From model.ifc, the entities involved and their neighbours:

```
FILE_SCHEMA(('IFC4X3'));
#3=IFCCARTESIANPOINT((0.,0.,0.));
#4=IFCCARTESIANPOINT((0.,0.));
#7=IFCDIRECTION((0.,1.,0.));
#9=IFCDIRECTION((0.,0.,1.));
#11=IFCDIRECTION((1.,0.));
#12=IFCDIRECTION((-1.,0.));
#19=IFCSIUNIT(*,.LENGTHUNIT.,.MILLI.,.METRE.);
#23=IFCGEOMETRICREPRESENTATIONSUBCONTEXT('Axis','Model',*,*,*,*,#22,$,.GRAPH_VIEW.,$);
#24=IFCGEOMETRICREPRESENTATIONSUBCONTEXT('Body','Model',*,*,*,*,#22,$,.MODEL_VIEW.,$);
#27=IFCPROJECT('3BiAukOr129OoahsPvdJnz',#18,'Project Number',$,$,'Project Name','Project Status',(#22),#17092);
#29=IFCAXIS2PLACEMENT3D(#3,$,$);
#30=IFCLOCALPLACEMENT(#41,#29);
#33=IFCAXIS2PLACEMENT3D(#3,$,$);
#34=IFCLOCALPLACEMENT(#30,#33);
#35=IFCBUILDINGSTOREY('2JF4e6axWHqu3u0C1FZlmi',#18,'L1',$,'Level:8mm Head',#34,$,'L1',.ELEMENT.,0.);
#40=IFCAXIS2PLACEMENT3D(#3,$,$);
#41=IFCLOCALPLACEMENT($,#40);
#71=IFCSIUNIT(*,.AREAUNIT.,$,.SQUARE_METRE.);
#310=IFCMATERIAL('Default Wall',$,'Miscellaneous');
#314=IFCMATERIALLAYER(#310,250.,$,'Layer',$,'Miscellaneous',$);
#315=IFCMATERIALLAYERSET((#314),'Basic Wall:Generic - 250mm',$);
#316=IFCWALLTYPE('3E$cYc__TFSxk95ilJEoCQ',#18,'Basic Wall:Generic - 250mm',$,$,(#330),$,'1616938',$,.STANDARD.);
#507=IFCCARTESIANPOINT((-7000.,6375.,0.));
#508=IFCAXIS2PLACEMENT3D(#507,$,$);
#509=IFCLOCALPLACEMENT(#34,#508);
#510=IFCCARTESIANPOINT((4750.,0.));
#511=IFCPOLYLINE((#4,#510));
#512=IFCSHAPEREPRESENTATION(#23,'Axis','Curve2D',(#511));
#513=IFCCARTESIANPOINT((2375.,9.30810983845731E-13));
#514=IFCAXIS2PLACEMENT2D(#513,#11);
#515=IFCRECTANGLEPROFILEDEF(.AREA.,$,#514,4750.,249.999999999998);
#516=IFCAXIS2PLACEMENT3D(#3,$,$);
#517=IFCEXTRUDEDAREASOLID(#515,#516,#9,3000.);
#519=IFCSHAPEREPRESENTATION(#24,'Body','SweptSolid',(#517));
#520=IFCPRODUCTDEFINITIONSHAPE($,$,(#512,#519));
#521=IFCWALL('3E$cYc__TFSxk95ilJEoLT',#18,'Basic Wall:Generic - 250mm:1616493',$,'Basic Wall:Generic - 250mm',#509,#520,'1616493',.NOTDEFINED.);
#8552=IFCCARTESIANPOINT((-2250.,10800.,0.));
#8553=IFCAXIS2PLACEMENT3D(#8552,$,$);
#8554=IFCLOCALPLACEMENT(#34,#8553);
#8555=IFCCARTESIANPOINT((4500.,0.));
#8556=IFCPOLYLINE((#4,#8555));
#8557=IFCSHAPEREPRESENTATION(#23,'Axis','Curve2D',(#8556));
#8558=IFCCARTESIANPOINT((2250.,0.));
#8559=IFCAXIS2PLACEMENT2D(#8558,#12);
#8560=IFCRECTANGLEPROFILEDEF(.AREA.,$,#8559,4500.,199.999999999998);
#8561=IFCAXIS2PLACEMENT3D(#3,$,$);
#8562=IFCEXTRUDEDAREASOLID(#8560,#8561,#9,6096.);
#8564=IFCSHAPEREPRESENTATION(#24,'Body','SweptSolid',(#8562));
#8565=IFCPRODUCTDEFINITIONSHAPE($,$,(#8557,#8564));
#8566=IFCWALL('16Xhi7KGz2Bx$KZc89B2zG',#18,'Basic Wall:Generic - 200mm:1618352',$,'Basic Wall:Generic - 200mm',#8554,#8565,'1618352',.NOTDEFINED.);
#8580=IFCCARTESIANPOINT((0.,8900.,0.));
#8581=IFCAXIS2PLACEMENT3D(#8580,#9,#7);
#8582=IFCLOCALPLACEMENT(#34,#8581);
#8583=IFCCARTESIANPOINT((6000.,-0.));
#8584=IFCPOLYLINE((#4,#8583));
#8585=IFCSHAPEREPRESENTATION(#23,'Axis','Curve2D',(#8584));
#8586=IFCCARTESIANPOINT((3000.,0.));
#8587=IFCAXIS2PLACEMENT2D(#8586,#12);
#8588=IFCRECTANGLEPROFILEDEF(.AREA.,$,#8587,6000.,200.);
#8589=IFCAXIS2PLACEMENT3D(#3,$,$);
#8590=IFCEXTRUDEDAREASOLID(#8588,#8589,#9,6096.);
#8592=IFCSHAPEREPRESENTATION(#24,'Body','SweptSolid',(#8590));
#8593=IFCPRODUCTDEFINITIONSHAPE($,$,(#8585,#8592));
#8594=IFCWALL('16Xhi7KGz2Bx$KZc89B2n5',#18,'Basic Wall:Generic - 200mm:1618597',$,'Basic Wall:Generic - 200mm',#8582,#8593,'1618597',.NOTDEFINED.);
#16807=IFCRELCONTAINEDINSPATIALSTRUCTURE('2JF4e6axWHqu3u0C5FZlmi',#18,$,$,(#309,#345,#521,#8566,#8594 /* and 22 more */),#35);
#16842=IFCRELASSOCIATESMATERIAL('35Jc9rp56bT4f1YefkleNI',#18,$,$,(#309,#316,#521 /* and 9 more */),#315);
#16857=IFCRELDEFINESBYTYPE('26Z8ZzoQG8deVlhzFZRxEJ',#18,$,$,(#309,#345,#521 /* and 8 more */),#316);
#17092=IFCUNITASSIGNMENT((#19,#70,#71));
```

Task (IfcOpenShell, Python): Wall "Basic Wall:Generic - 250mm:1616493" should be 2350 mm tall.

```python
import ifcopenshell
import ifcopenshell.geom
import ifcopenshell.util.representation
import ifcopenshell.util.shape
import ifcopenshell.util.unit

model = ifcopenshell.open("model.ifc")
unit_scale = ifcopenshell.util.unit.calculate_unit_scale(model)
settings = ifcopenshell.geom.settings()


def volume(element):
    """Net volume in cubic metres, openings subtracted."""
    shape = ifcopenshell.geom.create_shape(settings, element)
    return ifcopenshell.util.shape.get_volume(shape.geometry)


wall = model.by_guid("3E$cYc__TFSxk95ilJEoLT")
before = volume(wall)

body = ifcopenshell.util.representation.get_representation(wall, "Model", "Body")
solid = body.Items[0]
old_height = solid.Depth
solid.Depth = 2.35 / unit_scale
after = volume(wall)

print(f"height {old_height:g} -> {solid.Depth:g}, volume {before:.3f} -> {after:.3f} m3")

model.write("model_rev.ifc")
```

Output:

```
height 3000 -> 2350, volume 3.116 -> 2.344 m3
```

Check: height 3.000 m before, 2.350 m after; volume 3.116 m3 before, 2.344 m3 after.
